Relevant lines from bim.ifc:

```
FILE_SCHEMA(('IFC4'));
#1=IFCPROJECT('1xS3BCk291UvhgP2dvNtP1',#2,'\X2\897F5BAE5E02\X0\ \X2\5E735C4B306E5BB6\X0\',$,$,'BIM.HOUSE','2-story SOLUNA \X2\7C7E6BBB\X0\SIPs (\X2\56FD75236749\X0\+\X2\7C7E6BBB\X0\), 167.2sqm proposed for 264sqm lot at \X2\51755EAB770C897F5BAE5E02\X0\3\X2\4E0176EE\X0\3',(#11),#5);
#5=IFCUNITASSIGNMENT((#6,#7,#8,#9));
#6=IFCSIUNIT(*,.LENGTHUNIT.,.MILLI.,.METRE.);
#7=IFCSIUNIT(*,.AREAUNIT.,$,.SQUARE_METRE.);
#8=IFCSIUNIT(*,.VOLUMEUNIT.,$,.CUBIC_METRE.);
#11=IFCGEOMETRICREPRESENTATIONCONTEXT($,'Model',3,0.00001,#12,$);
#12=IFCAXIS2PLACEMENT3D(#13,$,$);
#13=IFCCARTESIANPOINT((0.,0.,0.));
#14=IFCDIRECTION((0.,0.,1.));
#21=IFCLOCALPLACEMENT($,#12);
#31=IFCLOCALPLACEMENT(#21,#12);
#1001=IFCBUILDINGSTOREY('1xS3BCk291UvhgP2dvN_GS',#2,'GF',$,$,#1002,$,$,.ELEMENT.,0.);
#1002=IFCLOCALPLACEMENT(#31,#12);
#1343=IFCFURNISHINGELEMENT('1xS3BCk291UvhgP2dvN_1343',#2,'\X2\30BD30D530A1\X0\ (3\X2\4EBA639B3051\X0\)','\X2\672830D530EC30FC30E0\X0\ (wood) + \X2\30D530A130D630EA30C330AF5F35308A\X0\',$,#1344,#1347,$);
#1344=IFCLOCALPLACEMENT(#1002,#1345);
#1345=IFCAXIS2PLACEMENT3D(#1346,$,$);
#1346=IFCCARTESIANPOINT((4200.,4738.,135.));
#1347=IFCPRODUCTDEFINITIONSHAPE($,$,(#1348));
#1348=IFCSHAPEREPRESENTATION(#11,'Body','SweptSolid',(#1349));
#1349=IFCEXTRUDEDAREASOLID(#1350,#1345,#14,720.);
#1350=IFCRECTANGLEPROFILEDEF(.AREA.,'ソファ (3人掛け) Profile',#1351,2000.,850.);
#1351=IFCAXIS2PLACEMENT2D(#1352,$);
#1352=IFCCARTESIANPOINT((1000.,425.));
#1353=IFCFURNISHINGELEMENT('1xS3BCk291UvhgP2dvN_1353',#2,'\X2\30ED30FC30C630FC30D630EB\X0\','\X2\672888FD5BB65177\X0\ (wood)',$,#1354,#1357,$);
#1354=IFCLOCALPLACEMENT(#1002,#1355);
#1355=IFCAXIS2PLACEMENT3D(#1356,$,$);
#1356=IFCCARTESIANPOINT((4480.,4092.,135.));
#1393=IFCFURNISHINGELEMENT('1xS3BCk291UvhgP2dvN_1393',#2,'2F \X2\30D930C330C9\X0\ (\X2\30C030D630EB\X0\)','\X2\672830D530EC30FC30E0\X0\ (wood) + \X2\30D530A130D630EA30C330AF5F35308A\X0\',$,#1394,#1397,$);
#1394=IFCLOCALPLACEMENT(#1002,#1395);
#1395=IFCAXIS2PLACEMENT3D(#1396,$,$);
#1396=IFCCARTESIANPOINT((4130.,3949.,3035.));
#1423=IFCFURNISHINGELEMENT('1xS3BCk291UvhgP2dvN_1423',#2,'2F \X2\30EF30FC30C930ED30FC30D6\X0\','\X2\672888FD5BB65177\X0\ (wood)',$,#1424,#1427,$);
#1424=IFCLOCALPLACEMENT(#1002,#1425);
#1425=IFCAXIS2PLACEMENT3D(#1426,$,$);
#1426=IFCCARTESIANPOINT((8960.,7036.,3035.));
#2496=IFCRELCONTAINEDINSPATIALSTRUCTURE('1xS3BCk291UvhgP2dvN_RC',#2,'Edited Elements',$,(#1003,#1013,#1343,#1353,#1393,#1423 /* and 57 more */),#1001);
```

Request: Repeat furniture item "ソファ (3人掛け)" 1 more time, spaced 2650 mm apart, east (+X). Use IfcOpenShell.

```python
import numpy as np
import ifcopenshell
import ifcopenshell.api.geometry
import ifcopenshell.api.root
import ifcopenshell.util.element
import ifcopenshell.util.placement

model = ifcopenshell.open("bim.ifc")


def reuse_history(source, copy):
    """copy_class also copies each property set's owner history, people and application; keep the originals."""
    for rel in copy.IsDefinedBy:
        if rel.is_a("IfcRelDefinesByProperties") and (history := rel.RelatingPropertyDefinition.OwnerHistory):
            rel.RelatingPropertyDefinition.OwnerHistory = source.OwnerHistory
            ifcopenshell.util.element.remove_deep2(model, history)


source = model.by_guid("1xS3BCk291UvhgP2dvN_1343")
base = ifcopenshell.util.placement.get_local_placement(source.ObjectPlacement)
step = np.array([1.0, 0.0, 0.0]) * 2650.0

for i in range(1, 2):
    copy = ifcopenshell.api.root.copy_class(model, product=source)
    copy.Representation = ifcopenshell.util.element.copy_deep(
        model, source.Representation, exclude=["IfcGeometricRepresentationContext", "IfcRepresentationMap"]
    )
    reuse_history(source, copy)
    matrix = base.copy()
    matrix[:3, 3] += i * step
    print("added at", matrix[:3, 3].round(3) + 0.0)
    ifcopenshell.api.geometry.edit_object_placement(model, product=copy, matrix=matrix, is_si=False)

model.write("bim_v2.ifc")
```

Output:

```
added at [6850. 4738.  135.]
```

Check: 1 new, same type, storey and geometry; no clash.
